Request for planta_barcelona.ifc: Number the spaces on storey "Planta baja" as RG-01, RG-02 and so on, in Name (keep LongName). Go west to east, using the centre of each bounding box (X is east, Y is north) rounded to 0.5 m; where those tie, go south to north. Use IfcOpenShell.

First a look at what the model holds.

```python
import ifcopenshell
import ifcopenshell.util.element
import ifcopenshell.util.placement

model = ifcopenshell.open("planta_barcelona.ifc")
print(model.schema)
storey = next(s for s in model.by_type("IfcBuildingStorey") if s.Name == "Planta baja")
spaces = [e for e in ifcopenshell.util.element.get_decomposition(storey) if e.is_a("IfcSpace")]
for e in sorted(spaces, key=lambda e: e.id()):
    origin = ifcopenshell.util.placement.get_local_placement(e.ObjectPlacement)[:3, 3]
    print(e.id(), e.Name, e.LongName, origin.round(2) + 0.0, sep=" | ")
```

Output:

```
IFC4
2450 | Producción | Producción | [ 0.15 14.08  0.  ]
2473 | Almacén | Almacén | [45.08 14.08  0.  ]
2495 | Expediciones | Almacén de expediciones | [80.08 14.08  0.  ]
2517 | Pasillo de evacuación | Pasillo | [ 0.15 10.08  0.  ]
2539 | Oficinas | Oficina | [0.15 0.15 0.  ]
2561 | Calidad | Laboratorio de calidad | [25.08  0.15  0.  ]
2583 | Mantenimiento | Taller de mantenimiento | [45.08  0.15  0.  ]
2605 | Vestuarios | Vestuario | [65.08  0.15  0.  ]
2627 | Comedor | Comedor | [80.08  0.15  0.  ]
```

```python
import ifcopenshell
import ifcopenshell.geom
import ifcopenshell.util.element
import ifcopenshell.util.shape

model = ifcopenshell.open("planta_barcelona.ifc")
settings = ifcopenshell.geom.settings()
settings.set("use-world-coords", True)


def centre(element):
    shape = ifcopenshell.geom.create_shape(settings, element)
    return ifcopenshell.util.shape.get_bbox_centroid(shape.geometry)


storey = next(s for s in model.by_type("IfcBuildingStorey") if s.Name == "Planta baja")
spaces = [e for e in ifcopenshell.util.element.get_decomposition(storey) if e.is_a("IfcSpace")]

# Insertion points can sit at a corner or the storey origin, so sort by the geometry (in metres).
centres = {e: centre(e) for e in spaces}
spaces.sort(key=lambda e: (round(centres[e][0] / 0.5), centres[e][1]))

for i, e in enumerate(spaces, start=1):
    number = f"RG-{i:02d}"
    e.Name = number
    print(e.id(), number)

model.write("planta_barcelona_v2.ifc")
```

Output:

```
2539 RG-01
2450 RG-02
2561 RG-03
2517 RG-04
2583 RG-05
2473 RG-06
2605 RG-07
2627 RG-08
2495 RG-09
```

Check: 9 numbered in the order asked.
